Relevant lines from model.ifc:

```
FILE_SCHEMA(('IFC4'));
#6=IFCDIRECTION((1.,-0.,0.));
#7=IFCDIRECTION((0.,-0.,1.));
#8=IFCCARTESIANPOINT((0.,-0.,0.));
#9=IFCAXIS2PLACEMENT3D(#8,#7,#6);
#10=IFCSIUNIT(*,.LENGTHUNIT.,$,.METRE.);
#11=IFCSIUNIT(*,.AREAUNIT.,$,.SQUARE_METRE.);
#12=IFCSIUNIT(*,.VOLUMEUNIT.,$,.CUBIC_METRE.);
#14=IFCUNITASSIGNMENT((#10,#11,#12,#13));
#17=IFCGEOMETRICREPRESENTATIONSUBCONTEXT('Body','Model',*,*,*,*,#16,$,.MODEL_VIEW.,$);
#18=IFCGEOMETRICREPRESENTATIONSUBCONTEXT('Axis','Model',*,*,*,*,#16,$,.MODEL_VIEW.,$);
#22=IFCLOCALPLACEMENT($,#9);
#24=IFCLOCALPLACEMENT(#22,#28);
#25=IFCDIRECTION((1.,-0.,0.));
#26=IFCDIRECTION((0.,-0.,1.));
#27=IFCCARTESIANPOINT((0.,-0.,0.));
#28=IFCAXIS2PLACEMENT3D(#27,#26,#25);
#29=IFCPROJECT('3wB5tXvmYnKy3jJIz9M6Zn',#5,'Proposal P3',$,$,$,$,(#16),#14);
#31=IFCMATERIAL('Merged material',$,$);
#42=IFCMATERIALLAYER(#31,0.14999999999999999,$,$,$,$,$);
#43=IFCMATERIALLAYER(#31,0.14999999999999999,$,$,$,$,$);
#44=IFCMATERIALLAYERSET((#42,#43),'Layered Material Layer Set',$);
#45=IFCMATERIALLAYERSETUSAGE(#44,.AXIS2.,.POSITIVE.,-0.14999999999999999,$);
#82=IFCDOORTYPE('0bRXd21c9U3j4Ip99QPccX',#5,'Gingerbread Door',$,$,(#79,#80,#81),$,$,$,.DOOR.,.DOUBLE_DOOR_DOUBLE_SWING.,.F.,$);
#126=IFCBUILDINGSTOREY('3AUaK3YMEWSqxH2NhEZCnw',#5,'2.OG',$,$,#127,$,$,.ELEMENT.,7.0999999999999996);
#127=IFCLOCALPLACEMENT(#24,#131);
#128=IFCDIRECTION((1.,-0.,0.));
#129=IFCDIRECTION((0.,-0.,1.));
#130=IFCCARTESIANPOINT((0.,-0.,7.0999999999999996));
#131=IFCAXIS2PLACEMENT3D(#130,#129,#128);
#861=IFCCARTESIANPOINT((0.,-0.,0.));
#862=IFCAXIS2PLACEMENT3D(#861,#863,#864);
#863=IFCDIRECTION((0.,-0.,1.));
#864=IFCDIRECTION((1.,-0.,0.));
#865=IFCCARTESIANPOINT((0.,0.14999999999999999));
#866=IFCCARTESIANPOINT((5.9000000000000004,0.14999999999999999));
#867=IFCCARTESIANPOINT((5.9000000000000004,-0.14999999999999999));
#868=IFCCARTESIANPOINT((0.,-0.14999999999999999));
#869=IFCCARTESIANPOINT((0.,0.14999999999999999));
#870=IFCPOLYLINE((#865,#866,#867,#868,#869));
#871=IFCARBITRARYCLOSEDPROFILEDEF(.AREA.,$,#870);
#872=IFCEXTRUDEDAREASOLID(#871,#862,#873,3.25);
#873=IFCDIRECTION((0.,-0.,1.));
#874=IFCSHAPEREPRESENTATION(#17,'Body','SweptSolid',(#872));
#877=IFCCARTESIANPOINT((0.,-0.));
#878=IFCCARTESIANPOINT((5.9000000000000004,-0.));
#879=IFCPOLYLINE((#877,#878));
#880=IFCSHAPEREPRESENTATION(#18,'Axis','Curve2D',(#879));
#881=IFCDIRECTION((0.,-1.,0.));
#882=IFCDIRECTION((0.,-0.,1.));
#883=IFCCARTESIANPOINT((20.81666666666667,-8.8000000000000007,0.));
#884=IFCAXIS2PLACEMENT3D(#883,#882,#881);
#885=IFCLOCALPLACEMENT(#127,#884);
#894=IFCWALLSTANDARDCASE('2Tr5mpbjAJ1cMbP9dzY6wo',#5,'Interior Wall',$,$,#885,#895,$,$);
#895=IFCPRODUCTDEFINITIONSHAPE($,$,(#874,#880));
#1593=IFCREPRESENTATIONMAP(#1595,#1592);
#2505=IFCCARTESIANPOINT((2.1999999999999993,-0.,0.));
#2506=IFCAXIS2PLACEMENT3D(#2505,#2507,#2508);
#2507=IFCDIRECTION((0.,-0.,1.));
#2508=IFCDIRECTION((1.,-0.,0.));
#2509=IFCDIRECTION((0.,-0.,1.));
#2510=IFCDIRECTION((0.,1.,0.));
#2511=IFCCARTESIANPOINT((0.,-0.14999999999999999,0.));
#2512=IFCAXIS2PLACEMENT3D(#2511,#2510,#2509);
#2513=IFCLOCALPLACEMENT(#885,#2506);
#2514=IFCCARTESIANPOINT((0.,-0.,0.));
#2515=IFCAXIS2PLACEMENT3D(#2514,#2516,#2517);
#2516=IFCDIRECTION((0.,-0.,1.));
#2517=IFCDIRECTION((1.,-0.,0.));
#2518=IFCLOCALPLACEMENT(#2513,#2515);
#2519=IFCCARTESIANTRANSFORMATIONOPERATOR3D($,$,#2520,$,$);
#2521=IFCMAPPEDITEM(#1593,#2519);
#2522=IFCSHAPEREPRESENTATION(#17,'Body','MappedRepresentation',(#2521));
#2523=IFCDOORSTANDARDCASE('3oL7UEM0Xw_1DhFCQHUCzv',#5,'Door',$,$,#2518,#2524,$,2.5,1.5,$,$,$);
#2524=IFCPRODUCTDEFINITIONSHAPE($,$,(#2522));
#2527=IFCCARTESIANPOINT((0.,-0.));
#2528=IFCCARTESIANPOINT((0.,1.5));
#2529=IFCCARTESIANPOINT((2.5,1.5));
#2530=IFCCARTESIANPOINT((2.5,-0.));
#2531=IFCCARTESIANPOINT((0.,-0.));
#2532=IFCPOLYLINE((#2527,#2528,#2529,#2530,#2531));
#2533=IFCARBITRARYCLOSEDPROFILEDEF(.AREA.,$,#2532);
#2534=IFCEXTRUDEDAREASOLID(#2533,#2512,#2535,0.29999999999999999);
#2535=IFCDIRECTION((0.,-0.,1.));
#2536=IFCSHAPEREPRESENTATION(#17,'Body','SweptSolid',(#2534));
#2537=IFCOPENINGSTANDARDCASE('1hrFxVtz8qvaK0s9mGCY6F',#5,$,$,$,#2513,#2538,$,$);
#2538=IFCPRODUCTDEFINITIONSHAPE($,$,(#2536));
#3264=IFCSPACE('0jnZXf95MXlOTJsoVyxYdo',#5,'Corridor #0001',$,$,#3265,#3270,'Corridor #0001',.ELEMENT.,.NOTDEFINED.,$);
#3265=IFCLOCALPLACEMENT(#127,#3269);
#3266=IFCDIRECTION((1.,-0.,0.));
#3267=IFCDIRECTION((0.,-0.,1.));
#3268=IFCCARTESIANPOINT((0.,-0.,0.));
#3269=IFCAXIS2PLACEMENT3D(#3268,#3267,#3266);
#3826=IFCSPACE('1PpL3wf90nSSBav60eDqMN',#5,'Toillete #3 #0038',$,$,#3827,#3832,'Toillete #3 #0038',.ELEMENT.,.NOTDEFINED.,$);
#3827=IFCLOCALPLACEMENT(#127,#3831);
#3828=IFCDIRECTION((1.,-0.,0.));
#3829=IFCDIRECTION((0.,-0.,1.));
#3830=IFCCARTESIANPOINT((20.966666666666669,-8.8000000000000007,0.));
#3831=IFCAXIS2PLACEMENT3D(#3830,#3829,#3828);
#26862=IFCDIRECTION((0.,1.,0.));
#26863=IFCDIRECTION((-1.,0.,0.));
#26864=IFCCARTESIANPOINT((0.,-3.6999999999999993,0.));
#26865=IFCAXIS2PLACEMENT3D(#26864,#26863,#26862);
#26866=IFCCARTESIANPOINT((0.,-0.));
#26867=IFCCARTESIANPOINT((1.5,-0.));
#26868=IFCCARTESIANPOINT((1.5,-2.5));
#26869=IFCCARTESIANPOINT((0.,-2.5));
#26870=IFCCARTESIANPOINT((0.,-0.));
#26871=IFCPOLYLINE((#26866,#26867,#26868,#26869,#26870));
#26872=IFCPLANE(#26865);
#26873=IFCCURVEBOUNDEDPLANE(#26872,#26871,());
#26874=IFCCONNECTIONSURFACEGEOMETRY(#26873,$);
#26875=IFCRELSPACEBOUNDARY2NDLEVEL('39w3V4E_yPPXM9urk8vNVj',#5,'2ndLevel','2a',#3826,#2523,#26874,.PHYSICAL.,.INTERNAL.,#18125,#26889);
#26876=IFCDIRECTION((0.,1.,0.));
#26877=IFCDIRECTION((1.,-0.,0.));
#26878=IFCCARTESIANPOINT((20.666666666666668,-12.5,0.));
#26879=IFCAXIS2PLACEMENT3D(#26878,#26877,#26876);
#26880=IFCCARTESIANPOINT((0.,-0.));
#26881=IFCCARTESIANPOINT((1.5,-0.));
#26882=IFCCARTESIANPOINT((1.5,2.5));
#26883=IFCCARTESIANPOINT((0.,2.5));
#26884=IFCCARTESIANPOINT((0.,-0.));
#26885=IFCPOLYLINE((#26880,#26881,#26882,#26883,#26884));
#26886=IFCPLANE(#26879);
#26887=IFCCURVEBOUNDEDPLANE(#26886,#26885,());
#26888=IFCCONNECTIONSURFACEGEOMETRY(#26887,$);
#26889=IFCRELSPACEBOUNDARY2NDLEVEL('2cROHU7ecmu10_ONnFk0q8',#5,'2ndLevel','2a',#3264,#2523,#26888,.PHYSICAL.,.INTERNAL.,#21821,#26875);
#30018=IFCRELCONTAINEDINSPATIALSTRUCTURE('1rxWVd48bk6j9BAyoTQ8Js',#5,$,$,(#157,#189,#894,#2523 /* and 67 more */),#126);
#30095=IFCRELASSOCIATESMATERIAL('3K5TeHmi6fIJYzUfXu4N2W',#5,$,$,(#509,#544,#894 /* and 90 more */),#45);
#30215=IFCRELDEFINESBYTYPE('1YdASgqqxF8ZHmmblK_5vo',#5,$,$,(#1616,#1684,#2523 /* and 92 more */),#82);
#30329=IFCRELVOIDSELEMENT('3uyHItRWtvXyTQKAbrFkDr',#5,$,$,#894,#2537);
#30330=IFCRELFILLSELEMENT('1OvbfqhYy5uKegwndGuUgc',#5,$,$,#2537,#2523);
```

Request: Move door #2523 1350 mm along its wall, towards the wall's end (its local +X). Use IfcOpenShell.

```python
import numpy as np
import ifcopenshell
import ifcopenshell.api.geometry
import ifcopenshell.util.placement

model = ifcopenshell.open("model.ifc")

door = model.by_id(2523)
opening = door.FillsVoids[0].RelatingOpeningElement
wall = opening.VoidsElements[0].RelatingBuildingElement

wall_matrix = ifcopenshell.util.placement.get_local_placement(wall.ObjectPlacement)
shift = wall_matrix[:3, 0] * 1.35
before = ifcopenshell.util.placement.get_local_placement(door.ObjectPlacement)[:3, 3].copy()

# The door is placed relative to its opening, so it follows when the opening moves.
matrix = ifcopenshell.util.placement.get_local_placement(opening.ObjectPlacement)
matrix[:3, 3] += shift
ifcopenshell.api.geometry.edit_object_placement(
    model, product=opening, matrix=matrix, is_si=False, should_transform_children=True
)

# Space boundary surfaces are stored in each space's coordinates; move them too.
for rel in door.ProvidesBoundaries:
    if not rel.ConnectionGeometry:
        continue
    surface = rel.ConnectionGeometry.SurfaceOnRelatingElement.BasisSurface
    space_matrix = ifcopenshell.util.placement.get_local_placement(rel.RelatingSpace.ObjectPlacement)
    point = np.array(surface.Position.Location.Coordinates) + space_matrix[:3, :3].T @ shift
    surface.Position = model.createIfcAxis2Placement3D(
        model.createIfcCartesianPoint(point.tolist()), surface.Position.Axis, surface.Position.RefDirection
    )

after = ifcopenshell.util.placement.get_local_placement(door.ObjectPlacement)[:3, 3]
print("door moved by", (after - before).round(3) + 0.0)

model.write("model_v2.ifc")
```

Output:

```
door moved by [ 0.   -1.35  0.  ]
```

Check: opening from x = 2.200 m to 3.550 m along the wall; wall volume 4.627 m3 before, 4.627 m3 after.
